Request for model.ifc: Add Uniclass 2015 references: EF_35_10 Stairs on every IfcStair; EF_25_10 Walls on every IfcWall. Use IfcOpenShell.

First a look at what the model holds.

```python
import ifcopenshell

model = ifcopenshell.open("model.ifc")
print(model.schema)
print("classifications:", [c.Name for c in model.by_type("IfcClassification")])
for ifc_class in ("IfcDoor", "IfcRoof", "IfcStair", "IfcWall", "IfcWindow"):
    print(ifc_class, len(model.by_type(ifc_class)))
```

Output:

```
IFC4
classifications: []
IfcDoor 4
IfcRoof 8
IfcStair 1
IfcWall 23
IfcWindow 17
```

```python
import ifcopenshell
import ifcopenshell.api.classification

model = ifcopenshell.open("model.ifc")

system = ifcopenshell.api.classification.add_classification(model, classification="Uniclass 2015")

codes = {
    "IfcStair": ("EF_35_10", "Stairs"),
    "IfcWall": ("EF_25_10", "Walls"),
}
for ifc_class, (code, name) in codes.items():
    products = model.by_type(ifc_class)
    ifcopenshell.api.classification.add_reference(
        model, products=products, classification=system, identification=code, name=name
    )
    print(code, len(products))

model.write("model-out.ifc")
```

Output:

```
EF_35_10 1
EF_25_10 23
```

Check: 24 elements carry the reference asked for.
